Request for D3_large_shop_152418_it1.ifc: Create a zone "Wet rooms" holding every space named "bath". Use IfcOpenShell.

First a look at what the model holds.

```python
import ifcopenshell

model = ifcopenshell.open("D3_large_shop_152418_it1.ifc")
print(model.schema)
seen = {}
for space in model.by_type("IfcSpace"):
    seen[space.LongName] = seen.get(space.LongName, 0) + 1
for name, count in sorted(seen.items(), key=str):
    print(count, "x", name)
print("zones:", [z.Name for z in model.by_type("IfcZone")][:20])
```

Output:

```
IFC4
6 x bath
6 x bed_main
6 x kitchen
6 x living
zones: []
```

```python
import ifcopenshell
import ifcopenshell.api.group
import ifcopenshell.api.root

model = ifcopenshell.open("D3_large_shop_152418_it1.ifc")

names = {"bath"}
spaces = [s for s in model.by_type("IfcSpace") if s.LongName in names]

zone = ifcopenshell.api.root.create_entity(model, ifc_class="IfcZone", name="Wet rooms")
ifcopenshell.api.group.assign_group(model, products=spaces, group=zone)
print(len(spaces), "spaces in", zone.Name)

model.write("D3_large_shop_152418_it1_updated.ifc")
```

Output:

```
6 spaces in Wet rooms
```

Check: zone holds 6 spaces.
